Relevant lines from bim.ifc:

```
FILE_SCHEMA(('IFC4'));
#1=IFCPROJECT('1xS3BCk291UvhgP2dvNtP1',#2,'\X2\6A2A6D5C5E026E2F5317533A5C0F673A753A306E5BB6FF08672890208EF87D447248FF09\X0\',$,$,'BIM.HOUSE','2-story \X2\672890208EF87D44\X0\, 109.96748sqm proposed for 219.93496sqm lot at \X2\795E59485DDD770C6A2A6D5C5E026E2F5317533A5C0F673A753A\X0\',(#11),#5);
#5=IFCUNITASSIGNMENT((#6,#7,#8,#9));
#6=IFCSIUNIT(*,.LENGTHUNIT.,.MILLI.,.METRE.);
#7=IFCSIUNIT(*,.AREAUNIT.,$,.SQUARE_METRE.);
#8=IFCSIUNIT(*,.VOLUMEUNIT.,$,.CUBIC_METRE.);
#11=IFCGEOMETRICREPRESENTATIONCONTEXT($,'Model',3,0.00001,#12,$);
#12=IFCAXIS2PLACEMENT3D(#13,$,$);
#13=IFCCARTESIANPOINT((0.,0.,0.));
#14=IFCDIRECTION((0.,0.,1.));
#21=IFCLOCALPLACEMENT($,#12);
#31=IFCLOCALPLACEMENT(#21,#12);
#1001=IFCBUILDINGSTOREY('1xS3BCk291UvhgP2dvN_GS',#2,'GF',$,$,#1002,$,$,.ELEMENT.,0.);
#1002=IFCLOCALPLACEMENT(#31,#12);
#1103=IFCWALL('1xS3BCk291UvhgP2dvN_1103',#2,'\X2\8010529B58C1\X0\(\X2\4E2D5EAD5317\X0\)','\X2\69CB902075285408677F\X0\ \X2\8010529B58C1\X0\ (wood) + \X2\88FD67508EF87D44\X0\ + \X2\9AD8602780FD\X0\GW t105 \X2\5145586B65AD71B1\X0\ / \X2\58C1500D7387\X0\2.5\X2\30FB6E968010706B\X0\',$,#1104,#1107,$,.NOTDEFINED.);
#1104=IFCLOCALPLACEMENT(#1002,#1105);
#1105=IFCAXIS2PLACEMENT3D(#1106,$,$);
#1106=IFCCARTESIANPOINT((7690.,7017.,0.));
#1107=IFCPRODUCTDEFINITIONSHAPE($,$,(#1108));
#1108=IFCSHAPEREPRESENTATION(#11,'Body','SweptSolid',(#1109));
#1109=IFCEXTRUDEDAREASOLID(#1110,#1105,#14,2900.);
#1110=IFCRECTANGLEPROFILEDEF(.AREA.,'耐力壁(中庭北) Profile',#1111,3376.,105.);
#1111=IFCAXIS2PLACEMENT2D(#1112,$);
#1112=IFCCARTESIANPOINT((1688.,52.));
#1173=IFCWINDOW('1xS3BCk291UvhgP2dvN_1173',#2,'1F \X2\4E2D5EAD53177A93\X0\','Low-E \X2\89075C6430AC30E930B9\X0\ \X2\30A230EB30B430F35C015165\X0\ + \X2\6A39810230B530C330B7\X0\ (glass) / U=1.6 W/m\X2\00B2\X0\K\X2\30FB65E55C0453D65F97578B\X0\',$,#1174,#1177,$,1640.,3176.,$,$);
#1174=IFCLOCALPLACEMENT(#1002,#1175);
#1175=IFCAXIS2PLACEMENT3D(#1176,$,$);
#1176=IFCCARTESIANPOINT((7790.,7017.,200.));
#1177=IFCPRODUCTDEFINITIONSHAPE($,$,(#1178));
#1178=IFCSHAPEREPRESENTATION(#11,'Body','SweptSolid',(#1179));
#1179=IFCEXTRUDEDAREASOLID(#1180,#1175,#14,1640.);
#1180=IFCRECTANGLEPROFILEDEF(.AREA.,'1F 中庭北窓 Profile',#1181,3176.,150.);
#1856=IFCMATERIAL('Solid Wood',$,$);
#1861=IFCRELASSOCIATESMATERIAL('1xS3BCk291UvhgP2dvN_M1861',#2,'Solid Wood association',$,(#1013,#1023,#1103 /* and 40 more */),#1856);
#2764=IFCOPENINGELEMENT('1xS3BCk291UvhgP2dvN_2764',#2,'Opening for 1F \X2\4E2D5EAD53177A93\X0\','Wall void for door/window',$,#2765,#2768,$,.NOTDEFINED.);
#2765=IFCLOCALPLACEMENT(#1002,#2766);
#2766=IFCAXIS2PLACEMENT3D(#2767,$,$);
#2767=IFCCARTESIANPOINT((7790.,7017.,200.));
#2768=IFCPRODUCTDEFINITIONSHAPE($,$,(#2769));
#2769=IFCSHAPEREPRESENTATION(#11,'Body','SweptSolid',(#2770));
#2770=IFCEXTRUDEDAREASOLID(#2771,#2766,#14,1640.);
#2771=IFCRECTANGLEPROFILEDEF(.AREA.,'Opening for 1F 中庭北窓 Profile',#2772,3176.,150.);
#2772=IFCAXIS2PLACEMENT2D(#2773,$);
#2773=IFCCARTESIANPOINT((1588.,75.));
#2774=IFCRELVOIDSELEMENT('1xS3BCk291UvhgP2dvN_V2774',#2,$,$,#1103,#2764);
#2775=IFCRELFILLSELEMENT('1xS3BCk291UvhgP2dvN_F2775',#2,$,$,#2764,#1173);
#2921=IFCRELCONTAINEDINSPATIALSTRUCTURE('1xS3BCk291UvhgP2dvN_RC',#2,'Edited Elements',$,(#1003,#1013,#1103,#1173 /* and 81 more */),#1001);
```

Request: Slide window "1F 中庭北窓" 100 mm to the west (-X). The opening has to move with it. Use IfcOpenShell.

```python
import ifcopenshell
import ifcopenshell.api.geometry
import ifcopenshell.util.placement

model = ifcopenshell.open("bim.ifc")

window = model.by_guid("1xS3BCk291UvhgP2dvN_1173")
opening = window.FillsVoids[0].RelatingOpeningElement
wall = opening.VoidsElements[0].RelatingBuildingElement

wall_matrix = ifcopenshell.util.placement.get_local_placement(wall.ObjectPlacement)
shift = wall_matrix[:3, 0] * -100.0
before = ifcopenshell.util.placement.get_local_placement(window.ObjectPlacement)[:3, 3].copy()

# The window is not placed relative to its opening, so move both.
for product in (opening, window):
    matrix = ifcopenshell.util.placement.get_local_placement(product.ObjectPlacement)
    matrix[:3, 3] += shift
    ifcopenshell.api.geometry.edit_object_placement(model, product=product, matrix=matrix, is_si=False)

after = ifcopenshell.util.placement.get_local_placement(window.ObjectPlacement)[:3, 3]
print("window moved by", (after - before).round(3) + 0.0)

model.write("bim_updated.ifc")
```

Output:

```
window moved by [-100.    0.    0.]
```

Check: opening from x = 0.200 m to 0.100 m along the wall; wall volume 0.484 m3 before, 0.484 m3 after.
